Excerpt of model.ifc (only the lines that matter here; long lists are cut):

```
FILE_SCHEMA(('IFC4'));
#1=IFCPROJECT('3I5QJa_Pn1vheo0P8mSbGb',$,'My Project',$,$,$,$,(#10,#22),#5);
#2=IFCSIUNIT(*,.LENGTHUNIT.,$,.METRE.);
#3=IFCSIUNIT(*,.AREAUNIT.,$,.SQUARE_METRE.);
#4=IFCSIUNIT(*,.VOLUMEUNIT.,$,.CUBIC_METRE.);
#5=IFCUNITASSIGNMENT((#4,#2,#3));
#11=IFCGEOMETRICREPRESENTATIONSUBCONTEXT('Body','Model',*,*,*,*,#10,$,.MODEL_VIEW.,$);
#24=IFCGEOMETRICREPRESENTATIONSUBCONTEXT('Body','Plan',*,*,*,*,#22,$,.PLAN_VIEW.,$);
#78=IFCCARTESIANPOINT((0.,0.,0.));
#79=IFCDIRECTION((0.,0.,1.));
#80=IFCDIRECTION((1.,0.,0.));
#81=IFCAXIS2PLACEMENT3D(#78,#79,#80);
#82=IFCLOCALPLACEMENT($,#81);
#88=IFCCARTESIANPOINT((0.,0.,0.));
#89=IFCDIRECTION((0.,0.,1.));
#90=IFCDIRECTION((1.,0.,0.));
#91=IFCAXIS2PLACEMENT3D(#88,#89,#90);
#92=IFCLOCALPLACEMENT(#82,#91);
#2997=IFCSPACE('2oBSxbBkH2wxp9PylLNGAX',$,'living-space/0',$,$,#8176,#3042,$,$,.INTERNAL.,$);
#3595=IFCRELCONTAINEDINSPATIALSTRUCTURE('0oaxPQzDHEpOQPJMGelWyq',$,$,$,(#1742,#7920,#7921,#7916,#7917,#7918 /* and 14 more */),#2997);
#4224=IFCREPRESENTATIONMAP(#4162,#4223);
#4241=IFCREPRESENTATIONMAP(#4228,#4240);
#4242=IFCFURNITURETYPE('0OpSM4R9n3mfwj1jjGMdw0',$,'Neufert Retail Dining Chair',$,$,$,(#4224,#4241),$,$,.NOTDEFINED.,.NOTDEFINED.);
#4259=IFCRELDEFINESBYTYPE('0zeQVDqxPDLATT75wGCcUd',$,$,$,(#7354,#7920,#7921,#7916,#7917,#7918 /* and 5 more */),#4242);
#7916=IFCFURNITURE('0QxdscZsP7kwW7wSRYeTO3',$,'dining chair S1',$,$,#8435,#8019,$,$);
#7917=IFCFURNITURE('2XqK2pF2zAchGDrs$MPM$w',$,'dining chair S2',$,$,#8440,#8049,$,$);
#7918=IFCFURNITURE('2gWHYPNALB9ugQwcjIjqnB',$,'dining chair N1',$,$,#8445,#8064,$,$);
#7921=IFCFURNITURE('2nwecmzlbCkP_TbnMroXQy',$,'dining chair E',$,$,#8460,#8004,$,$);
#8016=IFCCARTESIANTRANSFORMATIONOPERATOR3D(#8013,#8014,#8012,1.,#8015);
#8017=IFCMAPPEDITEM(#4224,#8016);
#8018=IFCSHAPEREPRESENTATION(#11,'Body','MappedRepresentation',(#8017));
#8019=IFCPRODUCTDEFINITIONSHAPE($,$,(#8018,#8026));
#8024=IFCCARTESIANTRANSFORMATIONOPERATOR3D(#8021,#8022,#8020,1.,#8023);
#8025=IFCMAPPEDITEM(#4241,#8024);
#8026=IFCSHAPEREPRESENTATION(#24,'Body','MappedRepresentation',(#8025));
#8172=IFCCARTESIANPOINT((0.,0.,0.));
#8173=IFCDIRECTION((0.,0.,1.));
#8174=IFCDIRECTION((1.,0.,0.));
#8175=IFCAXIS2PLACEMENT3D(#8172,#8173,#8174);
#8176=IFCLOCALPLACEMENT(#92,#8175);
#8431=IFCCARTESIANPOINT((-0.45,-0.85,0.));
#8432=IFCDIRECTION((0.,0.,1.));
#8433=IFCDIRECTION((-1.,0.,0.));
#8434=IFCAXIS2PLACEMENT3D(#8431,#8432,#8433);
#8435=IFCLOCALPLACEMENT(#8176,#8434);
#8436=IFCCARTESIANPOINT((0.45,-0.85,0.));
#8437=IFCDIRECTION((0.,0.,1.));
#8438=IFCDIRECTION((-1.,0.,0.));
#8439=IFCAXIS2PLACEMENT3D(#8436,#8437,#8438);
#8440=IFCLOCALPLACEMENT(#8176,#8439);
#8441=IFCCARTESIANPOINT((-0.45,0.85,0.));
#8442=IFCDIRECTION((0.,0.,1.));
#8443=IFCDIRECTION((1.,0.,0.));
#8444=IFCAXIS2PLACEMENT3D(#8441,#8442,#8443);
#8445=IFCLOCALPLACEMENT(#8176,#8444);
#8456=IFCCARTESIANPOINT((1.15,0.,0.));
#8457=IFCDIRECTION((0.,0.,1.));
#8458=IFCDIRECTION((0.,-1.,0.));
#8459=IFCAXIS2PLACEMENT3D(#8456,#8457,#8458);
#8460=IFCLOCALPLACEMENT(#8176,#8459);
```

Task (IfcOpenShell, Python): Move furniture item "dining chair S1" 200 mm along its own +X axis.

```python
import ifcopenshell
import ifcopenshell.api.geometry
import ifcopenshell.util.placement

model = ifcopenshell.open("model.ifc")

item = model.by_id(7916)
matrix = ifcopenshell.util.placement.get_local_placement(item.ObjectPlacement)
matrix[:3, 3] += matrix[:3, 0] * 0.2
ifcopenshell.api.geometry.edit_object_placement(model, product=item, matrix=matrix, is_si=False)

print(ifcopenshell.util.placement.get_local_placement(item.ObjectPlacement).round(3) + 0.0)

model.write("model_edited.ifc")
```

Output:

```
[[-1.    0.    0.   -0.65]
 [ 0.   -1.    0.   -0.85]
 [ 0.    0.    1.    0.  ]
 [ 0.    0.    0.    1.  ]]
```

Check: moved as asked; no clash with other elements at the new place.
